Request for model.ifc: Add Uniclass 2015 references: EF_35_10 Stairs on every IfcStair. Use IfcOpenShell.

First a look at what the model holds.

```python
import ifcopenshell

model = ifcopenshell.open("model.ifc")
print(model.schema)
print("classifications:", [c.Name for c in model.by_type("IfcClassification")])
for ifc_class in ("IfcDoor", "IfcRoof", "IfcStair", "IfcWall", "IfcWindow"):
    print(ifc_class, len(model.by_type(ifc_class)))
```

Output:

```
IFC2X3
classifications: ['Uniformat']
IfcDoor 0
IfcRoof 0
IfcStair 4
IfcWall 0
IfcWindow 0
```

```python
import ifcopenshell
import ifcopenshell.api.classification

model = ifcopenshell.open("model.ifc")

# IFC2X3 requires Source and Edition and has no link from the project to the system.
system = model.create_entity("IfcClassification", Source="NBS", Edition="2015", Name="Uniclass 2015")

codes = {
    "IfcStair": ("EF_35_10", "Stairs"),
}
for ifc_class, (code, name) in codes.items():
    products = model.by_type(ifc_class)
    ifcopenshell.api.classification.add_reference(
        model, products=products, classification=system, identification=code, name=name
    )
    print(code, len(products))

model.write("model_updated.ifc")
```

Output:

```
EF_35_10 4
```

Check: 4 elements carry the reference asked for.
